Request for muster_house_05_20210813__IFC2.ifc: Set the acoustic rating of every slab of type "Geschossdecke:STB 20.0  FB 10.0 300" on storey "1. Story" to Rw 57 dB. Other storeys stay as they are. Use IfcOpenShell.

First a look at what the model holds.

```python
import ifcopenshell
import ifcopenshell.util.element

model = ifcopenshell.open("muster_house_05_20210813__IFC2.ifc")
print(model.schema)
storey = next(s for s in model.by_type("IfcBuildingStorey") if s.Name == "1. Story")
slabs = [e for e in ifcopenshell.util.element.get_decomposition(storey) if e.is_a("IfcSlab")]
seen = {}
for e in slabs:
    element_type = ifcopenshell.util.element.get_type(e)
    key = (element_type.Name if element_type != e and element_type else None, ifcopenshell.util.element.get_pset(e, "Pset_SlabCommon", "AcousticRating"))
    seen[key] = seen.get(key, 0) + 1
for (name, value), count in sorted(seen.items(), key=str):
    print(count, "x", name, "|", value)
```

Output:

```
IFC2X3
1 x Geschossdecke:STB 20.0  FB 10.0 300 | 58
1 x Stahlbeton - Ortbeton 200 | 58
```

```python
import ifcopenshell
import ifcopenshell.api.pset
import ifcopenshell.util.element

model = ifcopenshell.open("muster_house_05_20210813__IFC2.ifc")

storey = next(s for s in model.by_type("IfcBuildingStorey") if s.Name == "1. Story")
slabs = [e for e in ifcopenshell.util.element.get_decomposition(storey) if e.is_a("IfcSlab")]

count = 0
for e in slabs:
    element_type = ifcopenshell.util.element.get_type(e)
    if element_type in (None, e) or element_type.Name != "Geschossdecke:STB 20.0  FB 10.0 300":
        continue
    # add_pset returns the element's existing set when there is one.
    pset = ifcopenshell.api.pset.add_pset(model, product=e, name="Pset_SlabCommon")
    ifcopenshell.api.pset.edit_pset(model, pset=pset, properties={"AcousticRating": "Rw 57 dB"})
    count += 1

print(count, "slabs updated")

model.write("muster_house_05_20210813__IFC2-out.ifc")
```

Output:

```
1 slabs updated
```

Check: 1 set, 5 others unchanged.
